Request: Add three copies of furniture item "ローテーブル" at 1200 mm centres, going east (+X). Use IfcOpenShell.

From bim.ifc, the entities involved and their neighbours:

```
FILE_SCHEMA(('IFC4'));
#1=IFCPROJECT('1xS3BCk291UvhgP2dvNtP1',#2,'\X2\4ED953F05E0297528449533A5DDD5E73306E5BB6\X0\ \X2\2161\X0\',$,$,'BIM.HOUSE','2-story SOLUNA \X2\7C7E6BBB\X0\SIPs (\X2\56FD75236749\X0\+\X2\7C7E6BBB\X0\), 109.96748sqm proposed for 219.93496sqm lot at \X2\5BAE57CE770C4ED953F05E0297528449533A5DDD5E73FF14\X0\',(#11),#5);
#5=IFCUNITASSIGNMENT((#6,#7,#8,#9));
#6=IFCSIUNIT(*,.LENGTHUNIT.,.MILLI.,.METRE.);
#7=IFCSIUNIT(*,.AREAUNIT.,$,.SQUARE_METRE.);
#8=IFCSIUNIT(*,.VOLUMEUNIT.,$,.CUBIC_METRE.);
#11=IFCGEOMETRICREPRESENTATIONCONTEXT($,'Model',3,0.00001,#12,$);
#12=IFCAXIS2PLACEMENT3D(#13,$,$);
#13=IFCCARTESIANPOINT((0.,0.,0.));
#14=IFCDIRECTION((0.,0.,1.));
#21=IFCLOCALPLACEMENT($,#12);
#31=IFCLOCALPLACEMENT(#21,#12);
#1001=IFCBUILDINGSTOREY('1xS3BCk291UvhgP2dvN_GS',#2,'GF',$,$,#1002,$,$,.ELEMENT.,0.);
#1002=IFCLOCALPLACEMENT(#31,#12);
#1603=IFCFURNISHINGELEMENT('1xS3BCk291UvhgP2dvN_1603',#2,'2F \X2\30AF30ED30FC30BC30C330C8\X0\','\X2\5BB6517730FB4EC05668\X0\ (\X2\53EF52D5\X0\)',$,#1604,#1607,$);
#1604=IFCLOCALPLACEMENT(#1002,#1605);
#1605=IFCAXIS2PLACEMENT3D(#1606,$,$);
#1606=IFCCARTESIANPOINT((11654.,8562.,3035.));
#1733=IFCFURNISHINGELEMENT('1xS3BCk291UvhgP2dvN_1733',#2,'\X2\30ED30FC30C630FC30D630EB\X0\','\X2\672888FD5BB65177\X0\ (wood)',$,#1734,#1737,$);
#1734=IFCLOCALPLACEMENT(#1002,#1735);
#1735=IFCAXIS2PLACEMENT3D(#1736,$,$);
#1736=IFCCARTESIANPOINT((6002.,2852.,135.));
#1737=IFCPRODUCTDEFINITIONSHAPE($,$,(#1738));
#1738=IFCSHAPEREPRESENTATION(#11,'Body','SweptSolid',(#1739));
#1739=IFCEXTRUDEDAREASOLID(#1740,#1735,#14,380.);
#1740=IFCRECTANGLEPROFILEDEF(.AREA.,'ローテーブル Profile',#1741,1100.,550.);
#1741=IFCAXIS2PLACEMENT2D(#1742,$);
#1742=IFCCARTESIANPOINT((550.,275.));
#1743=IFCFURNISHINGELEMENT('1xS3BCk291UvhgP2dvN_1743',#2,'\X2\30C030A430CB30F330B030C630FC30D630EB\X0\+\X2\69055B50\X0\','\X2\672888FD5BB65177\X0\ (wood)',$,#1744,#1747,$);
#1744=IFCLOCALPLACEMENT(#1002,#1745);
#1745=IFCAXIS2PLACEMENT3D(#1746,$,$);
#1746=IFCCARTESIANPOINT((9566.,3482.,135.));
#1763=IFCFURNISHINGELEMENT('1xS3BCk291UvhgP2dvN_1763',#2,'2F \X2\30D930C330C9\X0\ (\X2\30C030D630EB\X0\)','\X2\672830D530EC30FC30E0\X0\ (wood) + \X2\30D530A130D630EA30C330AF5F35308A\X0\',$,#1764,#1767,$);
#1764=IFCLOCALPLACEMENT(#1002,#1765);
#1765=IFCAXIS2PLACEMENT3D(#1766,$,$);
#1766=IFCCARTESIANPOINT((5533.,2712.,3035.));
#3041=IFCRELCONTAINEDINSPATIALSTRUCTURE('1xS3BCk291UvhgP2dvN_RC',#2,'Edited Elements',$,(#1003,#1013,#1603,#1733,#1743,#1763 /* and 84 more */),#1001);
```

```python
import numpy as np
import ifcopenshell
import ifcopenshell.api.geometry
import ifcopenshell.api.root
import ifcopenshell.util.element
import ifcopenshell.util.placement
import ifcopenshell.util.unit

model = ifcopenshell.open("bim.ifc")
unit_scale = ifcopenshell.util.unit.calculate_unit_scale(model)


def reuse_history(source, copy):
    """copy_class also copies each property set's owner history, people and application; keep the originals."""
    for rel in copy.IsDefinedBy:
        if rel.is_a("IfcRelDefinesByProperties") and (history := rel.RelatingPropertyDefinition.OwnerHistory):
            rel.RelatingPropertyDefinition.OwnerHistory = source.OwnerHistory
            ifcopenshell.util.element.remove_deep2(model, history)


source = model.by_guid("1xS3BCk291UvhgP2dvN_1733")
base = ifcopenshell.util.placement.get_local_placement(source.ObjectPlacement)
step = np.array([1.0, 0.0, 0.0]) * 1.2 / unit_scale

for i in range(1, 4):
    copy = ifcopenshell.api.root.copy_class(model, product=source)
    copy.Representation = ifcopenshell.util.element.copy_deep(
        model, source.Representation, exclude=["IfcGeometricRepresentationContext", "IfcRepresentationMap"]
    )
    reuse_history(source, copy)
    matrix = base.copy()
    matrix[:3, 3] += i * step
    print("added at", matrix[:3, 3].round(3) + 0.0)
    ifcopenshell.api.geometry.edit_object_placement(model, product=copy, matrix=matrix, is_si=False)

model.write("bim_rev.ifc")
```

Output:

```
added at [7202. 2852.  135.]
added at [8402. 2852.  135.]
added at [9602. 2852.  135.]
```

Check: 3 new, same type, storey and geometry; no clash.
